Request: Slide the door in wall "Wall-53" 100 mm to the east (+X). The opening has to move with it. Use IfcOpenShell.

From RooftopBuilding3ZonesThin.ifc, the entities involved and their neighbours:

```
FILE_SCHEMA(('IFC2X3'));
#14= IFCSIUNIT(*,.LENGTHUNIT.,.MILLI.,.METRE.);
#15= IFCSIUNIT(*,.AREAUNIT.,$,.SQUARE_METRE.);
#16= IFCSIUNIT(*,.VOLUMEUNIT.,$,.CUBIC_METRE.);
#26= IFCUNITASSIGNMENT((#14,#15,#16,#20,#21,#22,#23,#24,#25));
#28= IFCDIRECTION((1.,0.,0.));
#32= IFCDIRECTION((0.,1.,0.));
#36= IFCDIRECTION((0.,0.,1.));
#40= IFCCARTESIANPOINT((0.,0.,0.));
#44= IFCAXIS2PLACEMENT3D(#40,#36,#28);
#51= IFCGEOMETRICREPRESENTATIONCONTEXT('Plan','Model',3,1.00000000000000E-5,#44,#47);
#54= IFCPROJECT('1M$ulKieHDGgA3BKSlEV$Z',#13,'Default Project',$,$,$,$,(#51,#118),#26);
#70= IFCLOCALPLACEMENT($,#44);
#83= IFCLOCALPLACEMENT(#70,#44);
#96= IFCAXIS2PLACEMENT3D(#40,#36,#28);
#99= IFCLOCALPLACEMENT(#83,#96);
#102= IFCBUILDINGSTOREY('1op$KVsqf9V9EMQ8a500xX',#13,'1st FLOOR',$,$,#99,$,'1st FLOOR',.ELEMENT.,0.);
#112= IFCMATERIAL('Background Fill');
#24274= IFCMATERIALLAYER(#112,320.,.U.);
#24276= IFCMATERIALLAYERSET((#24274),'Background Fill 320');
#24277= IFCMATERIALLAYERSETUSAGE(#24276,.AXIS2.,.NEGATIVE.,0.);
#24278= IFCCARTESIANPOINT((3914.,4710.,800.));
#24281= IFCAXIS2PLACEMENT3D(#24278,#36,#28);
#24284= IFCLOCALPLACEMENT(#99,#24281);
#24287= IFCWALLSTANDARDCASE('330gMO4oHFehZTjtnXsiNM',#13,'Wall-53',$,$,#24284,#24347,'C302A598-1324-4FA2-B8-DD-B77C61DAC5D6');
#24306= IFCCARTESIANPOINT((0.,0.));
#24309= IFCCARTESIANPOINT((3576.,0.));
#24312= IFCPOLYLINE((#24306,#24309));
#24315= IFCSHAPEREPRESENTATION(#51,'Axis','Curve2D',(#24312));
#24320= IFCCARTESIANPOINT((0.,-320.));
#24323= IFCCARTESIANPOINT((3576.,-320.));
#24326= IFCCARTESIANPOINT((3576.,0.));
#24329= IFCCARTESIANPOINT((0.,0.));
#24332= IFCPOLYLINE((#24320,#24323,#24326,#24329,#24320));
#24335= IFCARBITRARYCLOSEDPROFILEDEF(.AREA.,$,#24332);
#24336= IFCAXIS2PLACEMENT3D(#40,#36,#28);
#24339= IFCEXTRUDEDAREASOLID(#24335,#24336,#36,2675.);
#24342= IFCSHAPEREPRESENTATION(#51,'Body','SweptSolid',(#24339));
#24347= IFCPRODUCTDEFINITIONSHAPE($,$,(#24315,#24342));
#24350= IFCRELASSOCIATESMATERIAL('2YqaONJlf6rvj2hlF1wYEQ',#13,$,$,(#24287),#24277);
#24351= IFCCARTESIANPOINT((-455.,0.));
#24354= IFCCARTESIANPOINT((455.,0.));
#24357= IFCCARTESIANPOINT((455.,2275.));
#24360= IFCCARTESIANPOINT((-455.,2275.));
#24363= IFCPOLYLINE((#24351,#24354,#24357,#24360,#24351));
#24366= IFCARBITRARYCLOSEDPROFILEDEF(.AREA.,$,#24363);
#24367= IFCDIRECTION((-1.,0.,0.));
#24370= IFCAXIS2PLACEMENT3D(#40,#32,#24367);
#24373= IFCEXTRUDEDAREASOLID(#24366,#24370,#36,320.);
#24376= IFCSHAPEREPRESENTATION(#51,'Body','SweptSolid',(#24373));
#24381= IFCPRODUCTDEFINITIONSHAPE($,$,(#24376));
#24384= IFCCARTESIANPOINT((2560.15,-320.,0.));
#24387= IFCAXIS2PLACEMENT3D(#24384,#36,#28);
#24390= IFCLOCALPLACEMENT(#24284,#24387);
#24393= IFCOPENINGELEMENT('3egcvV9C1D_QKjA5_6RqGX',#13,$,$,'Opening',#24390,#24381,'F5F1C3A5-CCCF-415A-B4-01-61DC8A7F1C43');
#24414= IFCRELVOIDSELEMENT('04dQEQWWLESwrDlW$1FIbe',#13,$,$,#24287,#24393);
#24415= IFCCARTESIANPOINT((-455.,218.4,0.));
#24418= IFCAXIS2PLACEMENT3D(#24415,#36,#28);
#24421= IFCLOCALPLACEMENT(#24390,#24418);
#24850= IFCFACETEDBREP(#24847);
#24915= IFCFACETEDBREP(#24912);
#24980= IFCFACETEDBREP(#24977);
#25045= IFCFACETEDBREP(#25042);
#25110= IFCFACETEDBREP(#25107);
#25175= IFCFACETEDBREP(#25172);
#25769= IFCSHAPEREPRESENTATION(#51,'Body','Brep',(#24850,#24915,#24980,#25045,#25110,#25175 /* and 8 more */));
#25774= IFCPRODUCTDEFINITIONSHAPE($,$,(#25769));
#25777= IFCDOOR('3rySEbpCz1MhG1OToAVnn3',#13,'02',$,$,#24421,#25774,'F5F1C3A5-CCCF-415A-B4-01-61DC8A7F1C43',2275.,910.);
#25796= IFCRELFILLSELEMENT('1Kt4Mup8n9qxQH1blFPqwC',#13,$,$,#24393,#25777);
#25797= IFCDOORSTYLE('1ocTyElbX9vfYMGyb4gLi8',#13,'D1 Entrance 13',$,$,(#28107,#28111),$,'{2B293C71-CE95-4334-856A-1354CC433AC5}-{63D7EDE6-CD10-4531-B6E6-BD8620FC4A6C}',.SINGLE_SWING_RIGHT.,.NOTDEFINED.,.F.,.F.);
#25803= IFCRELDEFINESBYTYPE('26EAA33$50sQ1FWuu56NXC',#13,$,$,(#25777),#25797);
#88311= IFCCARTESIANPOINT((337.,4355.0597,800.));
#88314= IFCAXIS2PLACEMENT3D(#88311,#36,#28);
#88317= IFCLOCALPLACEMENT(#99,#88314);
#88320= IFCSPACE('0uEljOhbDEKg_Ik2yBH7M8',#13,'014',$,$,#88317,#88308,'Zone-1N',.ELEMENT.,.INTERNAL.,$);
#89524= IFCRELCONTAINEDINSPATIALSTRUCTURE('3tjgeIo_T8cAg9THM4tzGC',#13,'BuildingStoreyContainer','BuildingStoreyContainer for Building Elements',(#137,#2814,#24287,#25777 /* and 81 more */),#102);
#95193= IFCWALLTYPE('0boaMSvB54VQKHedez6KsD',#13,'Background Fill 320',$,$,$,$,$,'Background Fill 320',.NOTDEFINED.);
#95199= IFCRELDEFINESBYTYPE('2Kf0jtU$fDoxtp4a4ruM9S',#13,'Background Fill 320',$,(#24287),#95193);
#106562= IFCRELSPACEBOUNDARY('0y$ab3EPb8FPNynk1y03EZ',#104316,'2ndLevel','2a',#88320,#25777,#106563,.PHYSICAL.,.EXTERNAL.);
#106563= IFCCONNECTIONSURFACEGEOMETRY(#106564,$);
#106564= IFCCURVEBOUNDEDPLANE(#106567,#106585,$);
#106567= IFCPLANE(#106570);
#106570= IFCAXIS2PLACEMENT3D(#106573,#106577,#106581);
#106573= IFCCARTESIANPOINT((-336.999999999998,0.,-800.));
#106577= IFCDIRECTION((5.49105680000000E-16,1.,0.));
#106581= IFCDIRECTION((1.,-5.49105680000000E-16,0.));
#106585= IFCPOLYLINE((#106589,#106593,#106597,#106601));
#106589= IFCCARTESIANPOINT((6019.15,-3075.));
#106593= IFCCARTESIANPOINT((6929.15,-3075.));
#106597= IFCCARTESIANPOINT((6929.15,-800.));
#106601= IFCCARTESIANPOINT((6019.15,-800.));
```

```python
import numpy as np
import ifcopenshell
import ifcopenshell.api.geometry
import ifcopenshell.util.placement

model = ifcopenshell.open("RooftopBuilding3ZonesThin.ifc")

door = model.by_guid("3rySEbpCz1MhG1OToAVnn3")
opening = door.FillsVoids[0].RelatingOpeningElement
wall = opening.VoidsElements[0].RelatingBuildingElement

wall_matrix = ifcopenshell.util.placement.get_local_placement(wall.ObjectPlacement)
shift = wall_matrix[:3, 0] * 100.0
before = ifcopenshell.util.placement.get_local_placement(door.ObjectPlacement)[:3, 3].copy()

# The door is placed relative to its opening, so it follows when the opening moves.
matrix = ifcopenshell.util.placement.get_local_placement(opening.ObjectPlacement)
matrix[:3, 3] += shift
ifcopenshell.api.geometry.edit_object_placement(
    model, product=opening, matrix=matrix, is_si=False, should_transform_children=True
)

# Space boundary surfaces are stored in each space's coordinates; move them too.
for rel in door.ProvidesBoundaries:
    if not rel.ConnectionGeometry:
        continue
    surface = rel.ConnectionGeometry.SurfaceOnRelatingElement.BasisSurface
    space_matrix = ifcopenshell.util.placement.get_local_placement(rel.RelatingSpace.ObjectPlacement)
    point = np.array(surface.Position.Location.Coordinates) + space_matrix[:3, :3].T @ shift
    surface.Position = model.createIfcAxis2Placement3D(
        model.createIfcCartesianPoint(point.tolist()), surface.Position.Axis, surface.Position.RefDirection
    )

after = ifcopenshell.util.placement.get_local_placement(door.ObjectPlacement)[:3, 3]
print("door moved by", (after - before).round(3) + 0.0)

model.write("RooftopBuilding3ZonesThin_edited.ifc")
```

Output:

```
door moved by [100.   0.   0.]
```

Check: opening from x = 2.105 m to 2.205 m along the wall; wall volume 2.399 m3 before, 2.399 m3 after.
